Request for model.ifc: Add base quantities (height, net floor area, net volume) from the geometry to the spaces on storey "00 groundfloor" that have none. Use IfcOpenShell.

First a look at what the model holds.

```python
import ifcopenshell
import ifcopenshell.util.element
import ifcopenshell.util.unit

model = ifcopenshell.open("model.ifc")
print(model.schema)
for unit_type in ("LENGTHUNIT", "AREAUNIT", "VOLUMEUNIT"):
    print(unit_type, ifcopenshell.util.unit.calculate_unit_scale(model, unit_type))
storey = next(s for s in model.by_type("IfcBuildingStorey") if s.Name == "00 groundfloor")
spaces = [e for e in ifcopenshell.util.element.get_decomposition(storey) if e.is_a("IfcSpace")]
for e in sorted(spaces, key=lambda e: e.id()):
    print(e.id(), e.is_a(), e.Name, list(ifcopenshell.util.element.get_psets(e, qtos_only=True)), sep=" | ")
```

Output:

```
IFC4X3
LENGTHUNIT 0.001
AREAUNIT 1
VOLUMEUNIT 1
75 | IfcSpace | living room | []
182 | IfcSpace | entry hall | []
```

```python
import ifcopenshell
import ifcopenshell.api.pset
import ifcopenshell.geom
import ifcopenshell.util.element
import ifcopenshell.util.shape
import ifcopenshell.util.unit

model = ifcopenshell.open("model.ifc")
unit_scale = ifcopenshell.util.unit.calculate_unit_scale(model)
area_scale = ifcopenshell.util.unit.calculate_unit_scale(model, "AREAUNIT")
volume_scale = ifcopenshell.util.unit.calculate_unit_scale(model, "VOLUMEUNIT")
settings = ifcopenshell.geom.settings()

storey = next(s for s in model.by_type("IfcBuildingStorey") if s.Name == "00 groundfloor")
spaces = [e for e in ifcopenshell.util.element.get_decomposition(storey) if e.is_a("IfcSpace")]

for e in sorted(spaces, key=lambda e: e.id()):
    if ifcopenshell.util.element.get_psets(e, qtos_only=True, should_inherit=False):
        continue
    # Geometry comes back in metres, in the element's own axes.
    shape = ifcopenshell.geom.create_shape(settings, e)
    values = {
        "Height": ifcopenshell.util.shape.get_z(shape.geometry) / unit_scale,
        "NetFloorArea": ifcopenshell.util.shape.get_footprint_area(shape.geometry) / area_scale,
        "NetVolume": ifcopenshell.util.shape.get_volume(shape.geometry) / volume_scale,
    }
    qto = ifcopenshell.api.pset.add_qto(model, product=e, name="Qto_SpaceBaseQuantities")
    ifcopenshell.api.pset.edit_qto(model, qto=qto, properties=values)
    print(e.id(), {k: round(v, 3) for k, v in values.items()})

model.write("model_edited.ifc")
```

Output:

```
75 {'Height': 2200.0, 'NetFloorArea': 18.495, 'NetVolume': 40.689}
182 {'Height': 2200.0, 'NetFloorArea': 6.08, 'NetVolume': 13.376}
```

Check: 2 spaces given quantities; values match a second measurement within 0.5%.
